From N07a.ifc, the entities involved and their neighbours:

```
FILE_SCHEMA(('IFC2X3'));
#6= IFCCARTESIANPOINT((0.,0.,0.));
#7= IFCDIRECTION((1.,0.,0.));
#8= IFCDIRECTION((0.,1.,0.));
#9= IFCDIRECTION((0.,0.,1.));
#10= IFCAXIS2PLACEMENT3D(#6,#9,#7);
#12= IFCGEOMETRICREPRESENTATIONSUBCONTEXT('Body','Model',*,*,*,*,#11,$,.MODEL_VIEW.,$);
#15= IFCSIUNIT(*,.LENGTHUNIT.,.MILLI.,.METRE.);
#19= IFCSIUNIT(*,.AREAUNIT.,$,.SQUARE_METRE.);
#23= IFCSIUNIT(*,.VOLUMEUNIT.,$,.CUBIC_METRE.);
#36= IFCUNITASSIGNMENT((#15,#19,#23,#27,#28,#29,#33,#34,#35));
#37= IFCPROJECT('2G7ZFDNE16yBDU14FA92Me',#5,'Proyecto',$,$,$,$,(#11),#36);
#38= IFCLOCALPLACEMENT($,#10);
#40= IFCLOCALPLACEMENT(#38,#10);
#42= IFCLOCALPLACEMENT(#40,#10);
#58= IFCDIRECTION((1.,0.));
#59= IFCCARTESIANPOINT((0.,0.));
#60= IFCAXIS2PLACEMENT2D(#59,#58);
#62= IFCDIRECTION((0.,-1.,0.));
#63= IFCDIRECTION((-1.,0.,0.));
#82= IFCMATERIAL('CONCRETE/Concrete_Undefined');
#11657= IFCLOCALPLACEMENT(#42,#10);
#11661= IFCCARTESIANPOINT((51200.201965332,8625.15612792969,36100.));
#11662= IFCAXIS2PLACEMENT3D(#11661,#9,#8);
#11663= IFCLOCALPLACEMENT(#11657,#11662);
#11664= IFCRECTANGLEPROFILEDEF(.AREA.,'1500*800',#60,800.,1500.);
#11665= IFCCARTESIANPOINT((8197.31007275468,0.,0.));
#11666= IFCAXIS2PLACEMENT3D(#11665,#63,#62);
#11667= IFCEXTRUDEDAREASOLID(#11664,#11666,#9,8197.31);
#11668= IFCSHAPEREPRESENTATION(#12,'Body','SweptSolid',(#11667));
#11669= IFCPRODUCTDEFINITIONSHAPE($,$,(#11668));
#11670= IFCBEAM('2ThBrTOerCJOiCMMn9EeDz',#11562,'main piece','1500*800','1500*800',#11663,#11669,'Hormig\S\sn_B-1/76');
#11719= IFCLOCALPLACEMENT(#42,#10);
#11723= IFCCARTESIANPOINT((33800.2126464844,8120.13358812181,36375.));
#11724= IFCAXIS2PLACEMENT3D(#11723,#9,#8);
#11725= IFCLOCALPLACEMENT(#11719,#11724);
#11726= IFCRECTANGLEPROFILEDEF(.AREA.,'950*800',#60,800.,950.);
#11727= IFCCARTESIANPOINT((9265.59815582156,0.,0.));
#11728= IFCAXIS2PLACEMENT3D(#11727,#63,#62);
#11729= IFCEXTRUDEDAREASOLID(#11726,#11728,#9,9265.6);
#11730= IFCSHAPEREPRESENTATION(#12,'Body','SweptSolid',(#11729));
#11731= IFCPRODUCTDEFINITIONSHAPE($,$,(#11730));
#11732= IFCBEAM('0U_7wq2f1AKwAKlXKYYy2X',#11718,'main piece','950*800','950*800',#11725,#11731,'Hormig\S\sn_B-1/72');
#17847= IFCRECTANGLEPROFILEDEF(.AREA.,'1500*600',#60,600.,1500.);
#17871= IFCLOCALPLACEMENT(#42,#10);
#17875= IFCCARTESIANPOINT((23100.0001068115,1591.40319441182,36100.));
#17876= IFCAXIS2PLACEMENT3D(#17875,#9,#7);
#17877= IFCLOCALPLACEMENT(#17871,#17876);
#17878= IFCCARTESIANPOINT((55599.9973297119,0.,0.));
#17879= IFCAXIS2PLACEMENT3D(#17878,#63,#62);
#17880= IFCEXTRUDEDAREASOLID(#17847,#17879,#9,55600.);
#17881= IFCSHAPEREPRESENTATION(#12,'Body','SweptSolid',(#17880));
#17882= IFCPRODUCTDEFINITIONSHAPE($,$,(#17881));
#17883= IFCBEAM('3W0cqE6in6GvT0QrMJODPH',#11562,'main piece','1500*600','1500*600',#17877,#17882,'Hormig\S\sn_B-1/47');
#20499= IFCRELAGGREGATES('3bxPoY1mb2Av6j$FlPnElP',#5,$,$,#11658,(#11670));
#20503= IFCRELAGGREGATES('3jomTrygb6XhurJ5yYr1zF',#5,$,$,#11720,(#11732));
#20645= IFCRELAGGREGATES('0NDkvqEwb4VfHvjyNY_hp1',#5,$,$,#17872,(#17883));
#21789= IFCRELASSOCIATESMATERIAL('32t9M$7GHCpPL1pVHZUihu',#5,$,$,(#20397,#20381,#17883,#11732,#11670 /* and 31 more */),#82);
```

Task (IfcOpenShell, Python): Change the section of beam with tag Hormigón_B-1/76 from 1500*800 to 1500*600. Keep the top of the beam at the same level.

```python
import ifcopenshell
import ifcopenshell.util.element
import ifcopenshell.util.representation

model = ifcopenshell.open("N07a.ifc")

member = model.by_id(11670)
source = next(p for p in model.by_type("IfcRectangleProfileDef") if p.ProfileName == "1500*600")

body = ifcopenshell.util.representation.get_representation(member, "Model", "Body")
solid = body.Items[0]
old_profile = solid.SweptArea

# Copy the section's sizes but keep this member's own profile position.
profile = ifcopenshell.util.element.copy(model, source)
# Profiles are centred, so shift by half the change in depth to hold the top.
shift = (old_profile.YDim - profile.YDim) / 2
x, y = old_profile.Position.Location.Coordinates
up = (0.0, 1.0)  # upwards, in the solid's own plane
location = model.createIfcCartesianPoint((x + up[0] * shift, y + up[1] * shift))
profile.Position = model.createIfcAxis2Placement2D(location, old_profile.Position.RefDirection)
solid.SweptArea = profile
if not model.get_total_inverses(old_profile):
    ifcopenshell.util.element.remove_deep2(model, old_profile)
member.Description = member.Description.replace("1500*800", "1500*600")
member.ObjectType = member.ObjectType.replace("1500*800", "1500*600")

print(solid.SweptArea)

model.write("N07a_rev.ifc")
```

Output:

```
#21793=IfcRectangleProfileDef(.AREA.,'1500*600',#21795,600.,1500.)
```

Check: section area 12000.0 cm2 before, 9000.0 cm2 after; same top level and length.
